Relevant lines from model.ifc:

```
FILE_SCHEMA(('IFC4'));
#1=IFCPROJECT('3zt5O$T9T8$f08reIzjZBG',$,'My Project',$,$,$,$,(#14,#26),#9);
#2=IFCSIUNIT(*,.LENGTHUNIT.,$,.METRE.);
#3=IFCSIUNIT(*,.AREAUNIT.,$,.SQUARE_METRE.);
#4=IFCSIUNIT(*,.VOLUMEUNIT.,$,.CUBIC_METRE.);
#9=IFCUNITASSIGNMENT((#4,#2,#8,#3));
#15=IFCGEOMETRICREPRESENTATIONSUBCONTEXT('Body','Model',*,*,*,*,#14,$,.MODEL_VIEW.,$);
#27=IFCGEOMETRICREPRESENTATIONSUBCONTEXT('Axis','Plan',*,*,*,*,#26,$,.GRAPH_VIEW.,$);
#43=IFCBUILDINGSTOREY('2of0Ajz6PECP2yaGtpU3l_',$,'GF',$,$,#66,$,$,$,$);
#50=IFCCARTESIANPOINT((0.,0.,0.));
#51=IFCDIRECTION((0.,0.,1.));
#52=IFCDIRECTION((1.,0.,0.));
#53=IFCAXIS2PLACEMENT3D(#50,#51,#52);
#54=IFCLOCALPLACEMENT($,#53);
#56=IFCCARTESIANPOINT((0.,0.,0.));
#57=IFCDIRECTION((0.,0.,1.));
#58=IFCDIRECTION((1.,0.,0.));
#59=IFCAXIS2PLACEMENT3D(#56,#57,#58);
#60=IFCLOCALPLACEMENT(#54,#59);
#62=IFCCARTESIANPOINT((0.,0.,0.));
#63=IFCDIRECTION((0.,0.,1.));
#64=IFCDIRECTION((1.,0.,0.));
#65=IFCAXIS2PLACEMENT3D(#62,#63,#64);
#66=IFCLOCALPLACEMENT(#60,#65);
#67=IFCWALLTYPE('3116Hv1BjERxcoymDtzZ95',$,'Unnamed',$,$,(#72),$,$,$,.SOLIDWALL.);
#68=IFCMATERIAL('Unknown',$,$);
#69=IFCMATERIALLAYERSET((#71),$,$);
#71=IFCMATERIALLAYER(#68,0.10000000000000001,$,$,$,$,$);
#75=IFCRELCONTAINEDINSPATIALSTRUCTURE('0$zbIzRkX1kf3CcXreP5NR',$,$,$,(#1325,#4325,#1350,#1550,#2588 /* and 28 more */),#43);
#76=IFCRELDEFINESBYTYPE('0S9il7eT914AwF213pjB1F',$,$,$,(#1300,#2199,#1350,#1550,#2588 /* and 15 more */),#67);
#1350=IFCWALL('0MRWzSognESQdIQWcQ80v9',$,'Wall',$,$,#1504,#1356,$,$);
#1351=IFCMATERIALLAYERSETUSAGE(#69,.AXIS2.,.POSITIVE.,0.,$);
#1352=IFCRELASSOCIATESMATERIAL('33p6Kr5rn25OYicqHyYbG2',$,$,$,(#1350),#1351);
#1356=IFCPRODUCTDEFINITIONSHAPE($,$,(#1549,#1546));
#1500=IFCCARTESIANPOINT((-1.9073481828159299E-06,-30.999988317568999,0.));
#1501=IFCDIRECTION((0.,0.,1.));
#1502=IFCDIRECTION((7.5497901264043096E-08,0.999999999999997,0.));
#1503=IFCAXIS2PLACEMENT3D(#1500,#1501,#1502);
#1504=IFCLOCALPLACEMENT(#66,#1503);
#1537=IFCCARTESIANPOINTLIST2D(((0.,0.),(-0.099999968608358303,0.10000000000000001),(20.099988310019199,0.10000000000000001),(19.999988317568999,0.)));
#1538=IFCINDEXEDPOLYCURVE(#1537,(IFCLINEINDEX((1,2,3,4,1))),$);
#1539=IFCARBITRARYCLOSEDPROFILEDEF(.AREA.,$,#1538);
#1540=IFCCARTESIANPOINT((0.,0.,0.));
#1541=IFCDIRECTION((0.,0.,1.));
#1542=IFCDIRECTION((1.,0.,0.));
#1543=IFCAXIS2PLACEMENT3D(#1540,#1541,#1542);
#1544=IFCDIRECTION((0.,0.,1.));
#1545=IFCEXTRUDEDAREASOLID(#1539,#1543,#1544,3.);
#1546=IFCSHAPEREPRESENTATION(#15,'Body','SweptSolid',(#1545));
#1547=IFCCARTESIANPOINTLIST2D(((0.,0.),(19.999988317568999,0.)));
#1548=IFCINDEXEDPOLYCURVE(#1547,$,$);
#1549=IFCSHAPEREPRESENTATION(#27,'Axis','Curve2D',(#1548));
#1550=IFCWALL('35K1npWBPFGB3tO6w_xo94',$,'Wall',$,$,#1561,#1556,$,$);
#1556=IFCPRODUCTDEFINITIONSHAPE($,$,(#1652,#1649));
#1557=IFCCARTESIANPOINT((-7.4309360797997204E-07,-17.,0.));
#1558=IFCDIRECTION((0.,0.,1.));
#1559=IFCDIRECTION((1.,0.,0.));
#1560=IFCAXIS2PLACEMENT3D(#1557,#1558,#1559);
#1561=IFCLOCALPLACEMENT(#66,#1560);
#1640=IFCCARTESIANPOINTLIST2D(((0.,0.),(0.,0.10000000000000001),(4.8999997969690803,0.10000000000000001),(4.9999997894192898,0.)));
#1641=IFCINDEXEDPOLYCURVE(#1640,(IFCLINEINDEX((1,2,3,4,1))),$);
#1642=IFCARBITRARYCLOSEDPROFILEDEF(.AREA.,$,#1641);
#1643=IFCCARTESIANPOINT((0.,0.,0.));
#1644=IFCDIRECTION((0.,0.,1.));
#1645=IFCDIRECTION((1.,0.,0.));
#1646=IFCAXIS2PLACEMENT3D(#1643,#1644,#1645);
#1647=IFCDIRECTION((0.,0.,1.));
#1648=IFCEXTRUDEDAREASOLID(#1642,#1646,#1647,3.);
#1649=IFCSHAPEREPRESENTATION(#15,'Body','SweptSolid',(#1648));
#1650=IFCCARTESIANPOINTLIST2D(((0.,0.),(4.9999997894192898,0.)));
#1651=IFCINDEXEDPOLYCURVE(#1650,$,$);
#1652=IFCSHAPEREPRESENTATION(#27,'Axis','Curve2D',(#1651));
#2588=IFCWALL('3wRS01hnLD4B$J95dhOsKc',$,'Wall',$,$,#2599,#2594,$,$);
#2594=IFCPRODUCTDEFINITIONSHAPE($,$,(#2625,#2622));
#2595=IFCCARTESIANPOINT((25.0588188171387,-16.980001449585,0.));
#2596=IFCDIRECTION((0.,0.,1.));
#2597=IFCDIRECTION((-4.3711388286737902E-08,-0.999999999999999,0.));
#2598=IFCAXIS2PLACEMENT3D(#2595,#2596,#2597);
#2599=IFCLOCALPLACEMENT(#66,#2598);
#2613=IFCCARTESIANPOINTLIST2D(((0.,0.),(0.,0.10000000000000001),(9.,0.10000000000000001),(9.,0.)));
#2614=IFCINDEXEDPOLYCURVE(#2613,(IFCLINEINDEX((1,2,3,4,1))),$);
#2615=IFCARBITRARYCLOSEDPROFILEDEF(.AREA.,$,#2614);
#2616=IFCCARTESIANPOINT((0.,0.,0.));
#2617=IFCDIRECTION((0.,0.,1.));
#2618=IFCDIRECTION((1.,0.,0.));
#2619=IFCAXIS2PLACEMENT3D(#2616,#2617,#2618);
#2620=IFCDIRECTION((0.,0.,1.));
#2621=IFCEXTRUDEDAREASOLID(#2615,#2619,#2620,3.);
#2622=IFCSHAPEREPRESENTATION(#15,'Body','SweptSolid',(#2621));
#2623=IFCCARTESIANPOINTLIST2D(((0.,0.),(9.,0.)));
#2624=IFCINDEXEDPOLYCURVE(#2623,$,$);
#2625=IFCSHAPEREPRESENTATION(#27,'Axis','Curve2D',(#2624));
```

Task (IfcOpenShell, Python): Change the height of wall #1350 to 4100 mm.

```python
import ifcopenshell
import ifcopenshell.geom
import ifcopenshell.util.representation
import ifcopenshell.util.shape

model = ifcopenshell.open("model.ifc")
settings = ifcopenshell.geom.settings()


def volume(element):
    """Net volume in cubic metres, openings subtracted."""
    shape = ifcopenshell.geom.create_shape(settings, element)
    return ifcopenshell.util.shape.get_volume(shape.geometry)


wall = model.by_guid("0MRWzSognESQdIQWcQ80v9")
before = volume(wall)

body = ifcopenshell.util.representation.get_representation(wall, "Model", "Body")
solid = body.Items[0]
old_height = solid.Depth
solid.Depth = 4.1
after = volume(wall)

print(f"height {old_height:g} -> {solid.Depth:g}, volume {before:.3f} -> {after:.3f} m3")

model.write("model-out.ifc")
```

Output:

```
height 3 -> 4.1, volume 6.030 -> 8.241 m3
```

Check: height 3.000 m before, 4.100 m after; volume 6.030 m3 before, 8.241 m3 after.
